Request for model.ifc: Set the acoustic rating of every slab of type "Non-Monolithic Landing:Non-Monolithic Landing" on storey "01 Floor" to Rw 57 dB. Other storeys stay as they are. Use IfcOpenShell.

First a look at what the model holds.

```python
import ifcopenshell
import ifcopenshell.util.element

model = ifcopenshell.open("model.ifc")
print(model.schema)
storey = next(s for s in model.by_type("IfcBuildingStorey") if s.Name == "01 Floor")
slabs = [e for e in ifcopenshell.util.element.get_decomposition(storey) if e.is_a("IfcSlab")]
seen = {}
for e in slabs:
    element_type = ifcopenshell.util.element.get_type(e)
    key = (element_type.Name if element_type != e and element_type else None, ifcopenshell.util.element.get_pset(e, "Pset_SlabCommon", "AcousticRating"))
    seen[key] = seen.get(key, 0) + 1
for (name, value), count in sorted(seen.items(), key=str):
    print(count, "x", name, "|", value)
```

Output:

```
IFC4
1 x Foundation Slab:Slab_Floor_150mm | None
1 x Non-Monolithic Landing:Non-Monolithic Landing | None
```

```python
import ifcopenshell
import ifcopenshell.api.pset
import ifcopenshell.util.element

model = ifcopenshell.open("model.ifc")

storey = next(s for s in model.by_type("IfcBuildingStorey") if s.Name == "01 Floor")
slabs = [e for e in ifcopenshell.util.element.get_decomposition(storey) if e.is_a("IfcSlab")]

count = 0
for e in slabs:
    element_type = ifcopenshell.util.element.get_type(e)
    if element_type in (None, e) or element_type.Name != "Non-Monolithic Landing:Non-Monolithic Landing":
        continue
    # add_pset returns the element's existing set when there is one.
    pset = ifcopenshell.api.pset.add_pset(model, product=e, name="Pset_SlabCommon")
    ifcopenshell.api.pset.edit_pset(model, pset=pset, properties={"AcousticRating": "Rw 57 dB"})
    count += 1

print(count, "slabs updated")

model.write("model_edited.ifc")
```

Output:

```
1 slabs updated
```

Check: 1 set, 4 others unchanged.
